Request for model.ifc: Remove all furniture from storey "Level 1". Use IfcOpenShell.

First a look at what the model holds.

```python
import ifcopenshell
import ifcopenshell.util.element

model = ifcopenshell.open("model.ifc")
print(model.schema)
storey = next(s for s in model.by_type("IfcBuildingStorey") if s.Name == "Level 1")
furniture = [e for e in ifcopenshell.util.element.get_decomposition(storey) if e.is_a("IfcFurnishingElement")]
seen = {}
for e in furniture:
    element_type = ifcopenshell.util.element.get_type(e)
    name = element_type.Name if element_type not in (None, e) else None
    seen[name] = seen.get(name, 0) + 1
for name, count in sorted(seen.items(), key=str):
    print(count, "x", name)
```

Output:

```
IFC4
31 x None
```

```python
import ifcopenshell
import ifcopenshell.api.root
import ifcopenshell.util.element

model = ifcopenshell.open("model.ifc")

storey = next(s for s in model.by_type("IfcBuildingStorey") if s.Name == "Level 1")
furniture = [e for e in ifcopenshell.util.element.get_decomposition(storey) if e.is_a("IfcFurnishingElement")]

for e in furniture:
    ifcopenshell.api.root.remove_product(model, product=e)
print(len(furniture), "removed")

model.write("model-out.ifc")
```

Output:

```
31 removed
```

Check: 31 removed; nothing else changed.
